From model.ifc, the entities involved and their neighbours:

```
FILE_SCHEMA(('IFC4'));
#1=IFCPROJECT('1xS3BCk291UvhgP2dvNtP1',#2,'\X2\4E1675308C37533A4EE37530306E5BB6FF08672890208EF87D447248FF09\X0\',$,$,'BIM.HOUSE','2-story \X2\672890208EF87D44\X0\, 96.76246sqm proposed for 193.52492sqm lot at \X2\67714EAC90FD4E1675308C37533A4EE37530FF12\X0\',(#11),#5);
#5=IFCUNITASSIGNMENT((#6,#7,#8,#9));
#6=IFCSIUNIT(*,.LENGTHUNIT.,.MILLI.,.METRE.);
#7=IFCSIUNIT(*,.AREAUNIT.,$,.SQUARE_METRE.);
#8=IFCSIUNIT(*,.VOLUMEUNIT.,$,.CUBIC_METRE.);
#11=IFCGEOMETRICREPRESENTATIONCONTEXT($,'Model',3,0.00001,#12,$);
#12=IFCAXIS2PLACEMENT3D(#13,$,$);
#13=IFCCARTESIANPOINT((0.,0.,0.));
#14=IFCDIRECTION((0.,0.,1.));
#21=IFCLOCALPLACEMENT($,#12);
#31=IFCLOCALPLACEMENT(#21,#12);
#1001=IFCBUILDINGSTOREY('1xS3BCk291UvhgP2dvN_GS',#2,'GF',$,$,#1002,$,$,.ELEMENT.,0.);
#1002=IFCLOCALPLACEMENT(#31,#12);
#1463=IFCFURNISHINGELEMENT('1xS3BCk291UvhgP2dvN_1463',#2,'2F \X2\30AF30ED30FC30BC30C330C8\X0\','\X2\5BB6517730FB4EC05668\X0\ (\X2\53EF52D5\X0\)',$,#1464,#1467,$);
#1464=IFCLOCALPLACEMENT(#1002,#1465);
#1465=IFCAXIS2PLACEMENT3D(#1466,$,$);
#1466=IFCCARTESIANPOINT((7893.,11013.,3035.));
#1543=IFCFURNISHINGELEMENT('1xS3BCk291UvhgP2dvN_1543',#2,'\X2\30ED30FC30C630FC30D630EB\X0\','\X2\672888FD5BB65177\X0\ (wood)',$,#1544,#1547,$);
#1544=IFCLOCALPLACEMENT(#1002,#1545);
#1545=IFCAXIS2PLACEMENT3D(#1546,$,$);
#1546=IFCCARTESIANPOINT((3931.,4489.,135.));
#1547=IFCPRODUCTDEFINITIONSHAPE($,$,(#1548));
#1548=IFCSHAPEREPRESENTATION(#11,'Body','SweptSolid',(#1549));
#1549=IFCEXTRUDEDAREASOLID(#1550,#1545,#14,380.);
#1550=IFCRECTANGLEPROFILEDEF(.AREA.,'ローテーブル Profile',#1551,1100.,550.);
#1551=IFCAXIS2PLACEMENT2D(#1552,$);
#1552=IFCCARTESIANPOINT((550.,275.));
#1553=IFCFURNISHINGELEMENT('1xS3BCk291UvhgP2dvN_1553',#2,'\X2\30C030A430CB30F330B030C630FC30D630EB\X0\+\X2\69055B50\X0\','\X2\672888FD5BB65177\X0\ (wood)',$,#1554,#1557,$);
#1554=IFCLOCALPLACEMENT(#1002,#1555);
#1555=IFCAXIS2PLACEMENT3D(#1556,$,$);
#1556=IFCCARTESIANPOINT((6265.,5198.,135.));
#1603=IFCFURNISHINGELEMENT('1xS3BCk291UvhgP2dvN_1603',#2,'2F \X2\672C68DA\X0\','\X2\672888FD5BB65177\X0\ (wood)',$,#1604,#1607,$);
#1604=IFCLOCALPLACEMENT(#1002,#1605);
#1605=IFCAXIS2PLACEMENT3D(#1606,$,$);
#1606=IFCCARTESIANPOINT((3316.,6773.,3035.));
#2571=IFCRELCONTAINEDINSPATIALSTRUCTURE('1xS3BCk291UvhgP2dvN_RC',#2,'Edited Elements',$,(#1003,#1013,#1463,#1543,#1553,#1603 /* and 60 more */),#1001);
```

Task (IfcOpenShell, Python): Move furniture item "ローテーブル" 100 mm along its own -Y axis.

```python
import ifcopenshell
import ifcopenshell.api.geometry
import ifcopenshell.util.placement
import ifcopenshell.util.unit

model = ifcopenshell.open("model.ifc")
unit_scale = ifcopenshell.util.unit.calculate_unit_scale(model)

item = model.by_id(1543)
matrix = ifcopenshell.util.placement.get_local_placement(item.ObjectPlacement)
matrix[:3, 3] -= matrix[:3, 1] * 0.1 / unit_scale
ifcopenshell.api.geometry.edit_object_placement(model, product=item, matrix=matrix, is_si=False)

print(ifcopenshell.util.placement.get_local_placement(item.ObjectPlacement).round(3) + 0.0)

model.write("model_v2.ifc")
```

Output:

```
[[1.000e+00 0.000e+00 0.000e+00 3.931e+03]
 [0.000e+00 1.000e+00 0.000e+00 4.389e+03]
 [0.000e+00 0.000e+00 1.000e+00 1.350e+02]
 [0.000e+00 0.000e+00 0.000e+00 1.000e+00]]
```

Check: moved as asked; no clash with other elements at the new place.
